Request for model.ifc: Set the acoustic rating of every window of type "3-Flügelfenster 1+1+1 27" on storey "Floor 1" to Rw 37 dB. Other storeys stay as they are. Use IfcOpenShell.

First a look at what the model holds.

```python
import ifcopenshell
import ifcopenshell.util.element

model = ifcopenshell.open("model.ifc")
print(model.schema)
storey = next(s for s in model.by_type("IfcBuildingStorey") if s.Name == "Floor 1")
windows = [e for e in ifcopenshell.util.element.get_decomposition(storey) if e.is_a("IfcWindow")]
seen = {}
for e in windows:
    element_type = ifcopenshell.util.element.get_type(e)
    key = (element_type.Name if element_type != e and element_type else None, ifcopenshell.util.element.get_pset(e, "Pset_WindowCommon", "AcousticRating"))
    seen[key] = seen.get(key, 0) + 1
for (name, value), count in sorted(seen.items(), key=str):
    print(count, "x", name, "|", value)
```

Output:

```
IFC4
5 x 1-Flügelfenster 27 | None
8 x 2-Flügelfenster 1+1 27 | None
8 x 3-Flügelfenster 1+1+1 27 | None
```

```python
import ifcopenshell
import ifcopenshell.api.pset
import ifcopenshell.util.element

model = ifcopenshell.open("model.ifc")

storey = next(s for s in model.by_type("IfcBuildingStorey") if s.Name == "Floor 1")
windows = [e for e in ifcopenshell.util.element.get_decomposition(storey) if e.is_a("IfcWindow")]

count = 0
for e in windows:
    element_type = ifcopenshell.util.element.get_type(e)
    if element_type in (None, e) or element_type.Name != "3-Flügelfenster 1+1+1 27":
        continue
    # add_pset returns the element's existing set when there is one.
    pset = ifcopenshell.api.pset.add_pset(model, product=e, name="Pset_WindowCommon")
    ifcopenshell.api.pset.edit_pset(model, pset=pset, properties={"AcousticRating": "Rw 37 dB"})
    count += 1

print(count, "windows updated")

model.write("model_v2.ifc")
```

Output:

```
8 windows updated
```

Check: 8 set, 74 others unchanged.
